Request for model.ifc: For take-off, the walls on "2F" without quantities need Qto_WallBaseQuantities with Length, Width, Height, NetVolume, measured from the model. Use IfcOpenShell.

First a look at what the model holds.

```python
import ifcopenshell
import ifcopenshell.util.element
import ifcopenshell.util.unit

model = ifcopenshell.open("model.ifc")
print(model.schema)
for unit_type in ("LENGTHUNIT", "AREAUNIT", "VOLUMEUNIT"):
    print(unit_type, ifcopenshell.util.unit.calculate_unit_scale(model, unit_type))
storey = next(s for s in model.by_type("IfcBuildingStorey") if s.Name == "2F")
walls = [e for e in ifcopenshell.util.element.get_decomposition(storey) if e.is_a("IfcWall")]
for e in sorted(walls, key=lambda e: e.id()):
    print(e.id(), e.is_a(), e.Name, list(ifcopenshell.util.element.get_psets(e, qtos_only=True)), sep=" | ")
```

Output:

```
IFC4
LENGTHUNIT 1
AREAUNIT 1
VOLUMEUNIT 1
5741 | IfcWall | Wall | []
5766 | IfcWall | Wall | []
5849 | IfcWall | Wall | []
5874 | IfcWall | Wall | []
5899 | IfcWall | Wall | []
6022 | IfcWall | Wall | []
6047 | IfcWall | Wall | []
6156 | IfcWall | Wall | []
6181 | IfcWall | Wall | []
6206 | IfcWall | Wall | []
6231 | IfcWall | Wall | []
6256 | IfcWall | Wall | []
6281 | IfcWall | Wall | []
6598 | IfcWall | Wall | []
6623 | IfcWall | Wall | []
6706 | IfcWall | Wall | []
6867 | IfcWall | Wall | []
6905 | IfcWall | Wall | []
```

```python
import ifcopenshell
import ifcopenshell.api.pset
import ifcopenshell.geom
import ifcopenshell.util.element
import ifcopenshell.util.shape
import ifcopenshell.util.unit

model = ifcopenshell.open("model.ifc")
unit_scale = ifcopenshell.util.unit.calculate_unit_scale(model)
volume_scale = ifcopenshell.util.unit.calculate_unit_scale(model, "VOLUMEUNIT")
settings = ifcopenshell.geom.settings()

storey = next(s for s in model.by_type("IfcBuildingStorey") if s.Name == "2F")
walls = [e for e in ifcopenshell.util.element.get_decomposition(storey) if e.is_a("IfcWall")]

for e in sorted(walls, key=lambda e: e.id()):
    if ifcopenshell.util.element.get_psets(e, qtos_only=True, should_inherit=False):
        continue
    # Geometry comes back in metres, in the element's own axes.
    shape = ifcopenshell.geom.create_shape(settings, e)
    values = {
        "Length": ifcopenshell.util.shape.get_x(shape.geometry) / unit_scale,
        "Width": ifcopenshell.util.shape.get_y(shape.geometry) / unit_scale,
        "Height": ifcopenshell.util.shape.get_z(shape.geometry) / unit_scale,
        "NetVolume": ifcopenshell.util.shape.get_volume(shape.geometry) / volume_scale,
    }
    qto = ifcopenshell.api.pset.add_qto(model, product=e, name="Qto_WallBaseQuantities")
    ifcopenshell.api.pset.edit_qto(model, qto=qto, properties=values)
    print(e.id(), {k: round(v, 3) for k, v in values.items()})

model.write("model_rev.ifc")
```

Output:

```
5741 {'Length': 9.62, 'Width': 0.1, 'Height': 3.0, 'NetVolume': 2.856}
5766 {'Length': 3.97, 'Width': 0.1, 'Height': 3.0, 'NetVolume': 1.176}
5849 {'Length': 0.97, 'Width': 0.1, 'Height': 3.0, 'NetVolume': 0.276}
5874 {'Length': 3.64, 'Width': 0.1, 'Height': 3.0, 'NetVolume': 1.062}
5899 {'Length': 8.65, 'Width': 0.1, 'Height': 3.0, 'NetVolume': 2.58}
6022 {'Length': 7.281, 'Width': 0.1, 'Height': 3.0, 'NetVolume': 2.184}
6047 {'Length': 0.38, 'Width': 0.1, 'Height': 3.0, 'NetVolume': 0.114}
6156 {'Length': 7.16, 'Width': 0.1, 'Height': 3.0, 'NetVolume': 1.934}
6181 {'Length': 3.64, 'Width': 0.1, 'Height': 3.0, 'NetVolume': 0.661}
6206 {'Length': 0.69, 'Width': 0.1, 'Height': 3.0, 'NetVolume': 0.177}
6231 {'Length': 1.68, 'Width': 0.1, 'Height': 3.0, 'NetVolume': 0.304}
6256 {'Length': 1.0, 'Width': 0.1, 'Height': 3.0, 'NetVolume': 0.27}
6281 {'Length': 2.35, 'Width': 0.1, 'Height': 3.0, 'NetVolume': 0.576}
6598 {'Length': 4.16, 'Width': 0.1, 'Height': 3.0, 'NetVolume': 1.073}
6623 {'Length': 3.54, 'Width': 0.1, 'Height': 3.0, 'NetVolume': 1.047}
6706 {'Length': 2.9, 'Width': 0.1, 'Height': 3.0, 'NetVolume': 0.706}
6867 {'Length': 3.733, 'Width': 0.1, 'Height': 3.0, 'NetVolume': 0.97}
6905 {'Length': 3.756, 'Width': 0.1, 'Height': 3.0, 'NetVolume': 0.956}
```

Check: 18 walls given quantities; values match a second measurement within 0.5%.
